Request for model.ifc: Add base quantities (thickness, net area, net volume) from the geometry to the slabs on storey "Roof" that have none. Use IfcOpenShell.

First a look at what the model holds.

```python
import ifcopenshell
import ifcopenshell.util.element
import ifcopenshell.util.unit

model = ifcopenshell.open("model.ifc")
print(model.schema)
for unit_type in ("LENGTHUNIT", "AREAUNIT", "VOLUMEUNIT"):
    print(unit_type, ifcopenshell.util.unit.calculate_unit_scale(model, unit_type))
storey = next(s for s in model.by_type("IfcBuildingStorey") if s.Name == "Roof")
slabs = [e for e in ifcopenshell.util.element.get_decomposition(storey) if e.is_a("IfcSlab")]
for e in sorted(slabs, key=lambda e: e.id()):
    print(e.id(), e.is_a(), e.Name, list(ifcopenshell.util.element.get_psets(e, qtos_only=True)), sep=" | ")
```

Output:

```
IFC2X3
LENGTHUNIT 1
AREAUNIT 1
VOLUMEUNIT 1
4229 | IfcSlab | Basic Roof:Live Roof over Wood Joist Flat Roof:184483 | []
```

```python
import ifcopenshell
import ifcopenshell.api.pset
import ifcopenshell.geom
import ifcopenshell.util.element
import ifcopenshell.util.shape
import ifcopenshell.util.unit

model = ifcopenshell.open("model.ifc")
unit_scale = ifcopenshell.util.unit.calculate_unit_scale(model)
area_scale = ifcopenshell.util.unit.calculate_unit_scale(model, "AREAUNIT")
volume_scale = ifcopenshell.util.unit.calculate_unit_scale(model, "VOLUMEUNIT")
settings = ifcopenshell.geom.settings()

storey = next(s for s in model.by_type("IfcBuildingStorey") if s.Name == "Roof")
slabs = [e for e in ifcopenshell.util.element.get_decomposition(storey) if e.is_a("IfcSlab")]

for e in sorted(slabs, key=lambda e: e.id()):
    if ifcopenshell.util.element.get_psets(e, qtos_only=True, should_inherit=False):
        continue
    # Geometry comes back in metres, in the element's own axes.
    shape = ifcopenshell.geom.create_shape(settings, e)
    values = {
        "Width": ifcopenshell.util.shape.get_z(shape.geometry) / unit_scale,
        "NetArea": ifcopenshell.util.shape.get_footprint_area(shape.geometry) / area_scale,
        "NetVolume": ifcopenshell.util.shape.get_volume(shape.geometry) / volume_scale,
    }
    qto = ifcopenshell.api.pset.add_qto(model, product=e, name="BaseQuantities")
    ifcopenshell.api.pset.edit_qto(model, qto=qto, properties=values)
    print(e.id(), {k: round(v, 3) for k, v in values.items()})

model.write("model-out.ifc")
```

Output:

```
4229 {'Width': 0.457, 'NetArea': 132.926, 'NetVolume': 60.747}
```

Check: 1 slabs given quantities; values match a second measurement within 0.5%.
